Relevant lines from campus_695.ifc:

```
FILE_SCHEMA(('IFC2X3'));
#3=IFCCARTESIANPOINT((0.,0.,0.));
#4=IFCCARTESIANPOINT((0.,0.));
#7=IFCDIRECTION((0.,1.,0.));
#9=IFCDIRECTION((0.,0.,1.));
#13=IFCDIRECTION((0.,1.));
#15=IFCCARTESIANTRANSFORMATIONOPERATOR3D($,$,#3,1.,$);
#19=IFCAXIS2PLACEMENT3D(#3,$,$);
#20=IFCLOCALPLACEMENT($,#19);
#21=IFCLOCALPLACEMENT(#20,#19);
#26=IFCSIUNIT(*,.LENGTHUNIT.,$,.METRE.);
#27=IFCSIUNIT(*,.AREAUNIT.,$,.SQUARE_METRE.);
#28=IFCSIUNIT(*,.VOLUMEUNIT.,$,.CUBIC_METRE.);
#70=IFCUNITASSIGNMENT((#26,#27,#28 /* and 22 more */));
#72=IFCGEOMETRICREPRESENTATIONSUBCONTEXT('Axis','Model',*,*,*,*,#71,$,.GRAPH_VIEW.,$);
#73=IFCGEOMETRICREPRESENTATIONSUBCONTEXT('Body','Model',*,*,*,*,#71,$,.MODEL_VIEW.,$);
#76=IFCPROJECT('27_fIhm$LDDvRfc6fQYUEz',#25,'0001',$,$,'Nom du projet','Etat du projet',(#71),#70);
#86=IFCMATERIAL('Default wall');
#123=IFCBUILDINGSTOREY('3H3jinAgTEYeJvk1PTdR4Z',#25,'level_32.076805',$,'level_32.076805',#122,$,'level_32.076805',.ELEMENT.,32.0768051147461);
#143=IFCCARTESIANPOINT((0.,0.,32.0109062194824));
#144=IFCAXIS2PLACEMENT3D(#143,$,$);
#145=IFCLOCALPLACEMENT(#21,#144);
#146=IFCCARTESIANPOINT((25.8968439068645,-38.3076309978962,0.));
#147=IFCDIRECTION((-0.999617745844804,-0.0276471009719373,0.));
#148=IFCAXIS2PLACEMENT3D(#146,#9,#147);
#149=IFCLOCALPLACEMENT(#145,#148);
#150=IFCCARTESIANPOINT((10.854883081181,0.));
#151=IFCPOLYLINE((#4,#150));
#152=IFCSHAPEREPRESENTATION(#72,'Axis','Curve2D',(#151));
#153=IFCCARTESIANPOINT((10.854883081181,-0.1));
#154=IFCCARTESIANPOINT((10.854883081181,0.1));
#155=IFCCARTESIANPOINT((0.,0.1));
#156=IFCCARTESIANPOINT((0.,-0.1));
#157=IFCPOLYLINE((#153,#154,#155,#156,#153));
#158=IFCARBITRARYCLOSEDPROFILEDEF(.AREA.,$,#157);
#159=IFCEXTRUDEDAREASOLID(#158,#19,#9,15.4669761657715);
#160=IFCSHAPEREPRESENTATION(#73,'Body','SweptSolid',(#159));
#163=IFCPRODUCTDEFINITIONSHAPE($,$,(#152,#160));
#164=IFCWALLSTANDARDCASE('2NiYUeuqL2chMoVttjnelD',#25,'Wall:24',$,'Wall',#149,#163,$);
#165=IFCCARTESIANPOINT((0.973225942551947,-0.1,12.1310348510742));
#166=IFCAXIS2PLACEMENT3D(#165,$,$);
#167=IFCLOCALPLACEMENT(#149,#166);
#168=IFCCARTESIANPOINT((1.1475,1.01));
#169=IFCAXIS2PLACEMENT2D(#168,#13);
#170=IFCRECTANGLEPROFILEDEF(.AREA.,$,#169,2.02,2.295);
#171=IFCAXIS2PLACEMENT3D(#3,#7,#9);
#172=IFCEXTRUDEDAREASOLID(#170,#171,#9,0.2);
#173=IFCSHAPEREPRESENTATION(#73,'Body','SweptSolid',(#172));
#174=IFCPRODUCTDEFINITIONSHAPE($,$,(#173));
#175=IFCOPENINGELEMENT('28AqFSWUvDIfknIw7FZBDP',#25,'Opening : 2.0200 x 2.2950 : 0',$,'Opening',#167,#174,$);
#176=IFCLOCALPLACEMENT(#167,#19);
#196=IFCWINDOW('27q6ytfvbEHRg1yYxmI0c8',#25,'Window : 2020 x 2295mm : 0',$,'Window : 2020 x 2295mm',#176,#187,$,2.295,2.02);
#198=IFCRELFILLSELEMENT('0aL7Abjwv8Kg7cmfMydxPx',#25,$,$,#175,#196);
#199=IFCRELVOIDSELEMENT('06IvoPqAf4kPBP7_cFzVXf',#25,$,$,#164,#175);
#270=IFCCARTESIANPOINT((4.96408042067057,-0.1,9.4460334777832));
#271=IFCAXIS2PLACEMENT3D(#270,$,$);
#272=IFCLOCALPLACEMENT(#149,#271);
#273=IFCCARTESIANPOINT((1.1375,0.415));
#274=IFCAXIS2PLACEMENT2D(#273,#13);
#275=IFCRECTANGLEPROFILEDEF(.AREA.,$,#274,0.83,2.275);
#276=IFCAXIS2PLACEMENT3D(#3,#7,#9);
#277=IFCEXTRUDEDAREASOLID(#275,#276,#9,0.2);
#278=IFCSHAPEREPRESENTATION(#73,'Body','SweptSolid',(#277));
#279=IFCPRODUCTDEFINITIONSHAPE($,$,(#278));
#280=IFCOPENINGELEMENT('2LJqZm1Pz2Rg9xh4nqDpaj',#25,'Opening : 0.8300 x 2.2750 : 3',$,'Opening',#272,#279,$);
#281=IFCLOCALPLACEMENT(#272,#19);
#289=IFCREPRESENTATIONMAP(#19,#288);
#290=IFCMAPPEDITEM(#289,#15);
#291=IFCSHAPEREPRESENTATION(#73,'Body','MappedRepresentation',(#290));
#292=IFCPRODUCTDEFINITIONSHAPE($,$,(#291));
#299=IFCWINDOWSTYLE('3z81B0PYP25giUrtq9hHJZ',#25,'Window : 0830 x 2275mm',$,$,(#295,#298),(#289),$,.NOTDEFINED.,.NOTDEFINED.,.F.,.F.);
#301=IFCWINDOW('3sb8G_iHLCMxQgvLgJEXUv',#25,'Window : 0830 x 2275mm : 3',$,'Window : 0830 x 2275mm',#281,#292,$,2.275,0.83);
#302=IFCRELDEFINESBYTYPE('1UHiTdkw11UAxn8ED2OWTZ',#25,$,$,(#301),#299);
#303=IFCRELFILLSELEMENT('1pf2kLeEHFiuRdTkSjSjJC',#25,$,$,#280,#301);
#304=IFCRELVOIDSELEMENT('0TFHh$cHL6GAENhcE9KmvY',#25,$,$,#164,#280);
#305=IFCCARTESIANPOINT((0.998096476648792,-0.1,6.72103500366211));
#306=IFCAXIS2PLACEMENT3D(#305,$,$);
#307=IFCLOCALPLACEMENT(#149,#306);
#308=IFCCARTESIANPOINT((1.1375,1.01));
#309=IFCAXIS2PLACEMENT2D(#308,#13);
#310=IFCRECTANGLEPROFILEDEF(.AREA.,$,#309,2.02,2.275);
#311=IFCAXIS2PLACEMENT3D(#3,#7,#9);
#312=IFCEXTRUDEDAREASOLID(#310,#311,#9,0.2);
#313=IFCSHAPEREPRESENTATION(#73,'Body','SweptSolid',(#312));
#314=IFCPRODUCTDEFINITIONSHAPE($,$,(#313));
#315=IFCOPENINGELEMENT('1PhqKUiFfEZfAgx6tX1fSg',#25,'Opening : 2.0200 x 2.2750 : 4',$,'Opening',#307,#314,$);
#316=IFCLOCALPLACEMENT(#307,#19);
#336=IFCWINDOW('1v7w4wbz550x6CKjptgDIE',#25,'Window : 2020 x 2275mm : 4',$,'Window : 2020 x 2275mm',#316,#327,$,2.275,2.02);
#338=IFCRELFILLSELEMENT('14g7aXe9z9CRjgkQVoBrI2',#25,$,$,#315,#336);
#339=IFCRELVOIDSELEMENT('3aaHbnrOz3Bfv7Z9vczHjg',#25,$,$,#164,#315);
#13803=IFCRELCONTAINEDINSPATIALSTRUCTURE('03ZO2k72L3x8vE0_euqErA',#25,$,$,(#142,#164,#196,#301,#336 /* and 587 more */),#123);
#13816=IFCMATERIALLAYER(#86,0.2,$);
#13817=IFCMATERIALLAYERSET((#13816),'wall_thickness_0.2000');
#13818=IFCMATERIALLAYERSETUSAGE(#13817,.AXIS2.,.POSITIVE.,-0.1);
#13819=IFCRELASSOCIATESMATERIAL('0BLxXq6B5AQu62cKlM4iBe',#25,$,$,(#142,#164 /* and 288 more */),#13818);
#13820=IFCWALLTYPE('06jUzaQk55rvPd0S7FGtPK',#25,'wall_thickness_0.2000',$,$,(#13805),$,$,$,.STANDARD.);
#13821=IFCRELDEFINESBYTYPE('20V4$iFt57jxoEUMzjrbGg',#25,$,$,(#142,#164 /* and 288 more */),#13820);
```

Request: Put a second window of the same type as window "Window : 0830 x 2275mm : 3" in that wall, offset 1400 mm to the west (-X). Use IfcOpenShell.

```python
import ifcopenshell
import ifcopenshell.api.feature
import ifcopenshell.api.geometry
import ifcopenshell.api.root
import ifcopenshell.geom
import ifcopenshell.util.element
import ifcopenshell.util.placement
import ifcopenshell.util.shape

model = ifcopenshell.open("campus_695.ifc")
settings = ifcopenshell.geom.settings()


def volume(element):
    """Net volume in cubic metres, openings subtracted."""
    shape = ifcopenshell.geom.create_shape(settings, element)
    return ifcopenshell.util.shape.get_volume(shape.geometry)


window = model.by_guid("3sb8G_iHLCMxQgvLgJEXUv")
opening = window.FillsVoids[0].RelatingOpeningElement
wall = opening.VoidsElements[0].RelatingBuildingElement
before = volume(wall)
shift = ifcopenshell.util.placement.get_local_placement(wall.ObjectPlacement)[:3, 0] * 1.4

# copy_class copies the void relationship, type, container and properties, but no geometry.
new_opening = ifcopenshell.api.root.copy_class(model, product=opening)
new_opening.Representation = ifcopenshell.util.element.copy_deep(
    model, opening.Representation, exclude=["IfcGeometricRepresentationContext", "IfcRepresentationMap"]
)
new_opening.Name = "Opening : 0.8300 x 2.2750"
new_window = ifcopenshell.api.root.copy_class(model, product=window)
new_window.Representation = ifcopenshell.util.element.copy_deep(
    model, window.Representation, exclude=["IfcGeometricRepresentationContext", "IfcRepresentationMap"]
)
new_window.Name = "Window : 0830 x 2275mm"
fills = ifcopenshell.api.feature.add_filling(model, opening=new_opening, element=new_window)
fills.OwnerHistory = new_window.OwnerHistory  # required in IFC2X3

for old, new in ((opening, new_opening), (window, new_window)):
    matrix = ifcopenshell.util.placement.get_local_placement(old.ObjectPlacement)
    matrix[:3, 3] += shift
    ifcopenshell.api.geometry.edit_object_placement(model, product=new, matrix=matrix, is_si=False)

after = volume(wall)

print(f"wall volume {before:.3f} -> {after:.3f} m3")

model.write("campus_695-out.ifc")
```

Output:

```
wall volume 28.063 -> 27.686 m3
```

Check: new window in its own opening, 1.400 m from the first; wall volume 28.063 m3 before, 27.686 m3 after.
